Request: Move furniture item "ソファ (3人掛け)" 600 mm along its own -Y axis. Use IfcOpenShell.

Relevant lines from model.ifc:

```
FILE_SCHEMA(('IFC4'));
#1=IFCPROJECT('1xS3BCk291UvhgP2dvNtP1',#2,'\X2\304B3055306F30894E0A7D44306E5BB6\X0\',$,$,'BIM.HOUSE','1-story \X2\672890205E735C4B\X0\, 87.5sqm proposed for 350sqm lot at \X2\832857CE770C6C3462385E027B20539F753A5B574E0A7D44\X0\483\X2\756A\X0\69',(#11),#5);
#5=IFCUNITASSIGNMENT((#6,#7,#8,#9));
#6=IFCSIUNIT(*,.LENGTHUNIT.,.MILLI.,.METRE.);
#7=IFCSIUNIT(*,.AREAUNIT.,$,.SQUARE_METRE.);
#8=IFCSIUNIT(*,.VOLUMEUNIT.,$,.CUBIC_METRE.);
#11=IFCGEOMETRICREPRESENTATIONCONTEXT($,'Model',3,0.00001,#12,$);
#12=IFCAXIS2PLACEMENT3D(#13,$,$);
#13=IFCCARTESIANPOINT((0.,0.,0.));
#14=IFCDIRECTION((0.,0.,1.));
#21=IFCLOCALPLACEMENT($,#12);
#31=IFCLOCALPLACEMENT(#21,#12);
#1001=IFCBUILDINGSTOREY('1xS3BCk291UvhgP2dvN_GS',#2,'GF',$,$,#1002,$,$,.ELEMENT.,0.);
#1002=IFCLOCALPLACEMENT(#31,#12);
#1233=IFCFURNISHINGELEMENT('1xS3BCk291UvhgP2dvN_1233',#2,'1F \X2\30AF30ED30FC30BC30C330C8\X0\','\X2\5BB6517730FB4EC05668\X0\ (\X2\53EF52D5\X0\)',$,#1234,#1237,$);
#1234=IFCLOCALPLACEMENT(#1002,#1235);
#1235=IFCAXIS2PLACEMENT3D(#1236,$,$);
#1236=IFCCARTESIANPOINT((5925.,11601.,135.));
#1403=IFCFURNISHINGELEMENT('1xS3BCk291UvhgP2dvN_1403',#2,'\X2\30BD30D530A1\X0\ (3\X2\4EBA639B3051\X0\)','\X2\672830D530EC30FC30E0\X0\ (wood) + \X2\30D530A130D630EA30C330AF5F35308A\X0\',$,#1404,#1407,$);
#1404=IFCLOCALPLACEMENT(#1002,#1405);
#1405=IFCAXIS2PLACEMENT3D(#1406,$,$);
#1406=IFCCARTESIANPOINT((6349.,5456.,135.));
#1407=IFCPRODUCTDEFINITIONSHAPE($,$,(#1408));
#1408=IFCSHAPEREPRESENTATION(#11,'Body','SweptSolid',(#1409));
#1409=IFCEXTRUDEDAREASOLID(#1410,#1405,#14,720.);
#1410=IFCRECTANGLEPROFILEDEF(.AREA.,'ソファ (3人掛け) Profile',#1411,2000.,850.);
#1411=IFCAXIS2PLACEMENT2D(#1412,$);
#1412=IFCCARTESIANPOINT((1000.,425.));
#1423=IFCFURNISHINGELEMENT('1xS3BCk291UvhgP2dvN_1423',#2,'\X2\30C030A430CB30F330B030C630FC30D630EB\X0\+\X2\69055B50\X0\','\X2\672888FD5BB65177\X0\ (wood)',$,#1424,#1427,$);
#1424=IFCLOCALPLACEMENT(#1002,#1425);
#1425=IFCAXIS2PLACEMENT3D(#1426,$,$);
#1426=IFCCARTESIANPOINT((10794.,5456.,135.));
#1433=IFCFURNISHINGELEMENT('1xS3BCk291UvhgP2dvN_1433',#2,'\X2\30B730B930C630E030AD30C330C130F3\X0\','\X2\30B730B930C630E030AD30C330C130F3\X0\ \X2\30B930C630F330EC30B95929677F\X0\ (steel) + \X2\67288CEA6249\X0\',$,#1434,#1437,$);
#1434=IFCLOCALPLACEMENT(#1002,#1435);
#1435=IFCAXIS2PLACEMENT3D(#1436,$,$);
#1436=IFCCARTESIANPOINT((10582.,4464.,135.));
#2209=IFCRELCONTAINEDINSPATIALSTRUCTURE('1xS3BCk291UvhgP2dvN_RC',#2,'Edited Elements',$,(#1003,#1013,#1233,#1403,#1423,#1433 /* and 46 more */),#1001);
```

```python
import ifcopenshell
import ifcopenshell.api.geometry
import ifcopenshell.util.placement
import ifcopenshell.util.unit

model = ifcopenshell.open("model.ifc")
unit_scale = ifcopenshell.util.unit.calculate_unit_scale(model)

item = model.by_guid("1xS3BCk291UvhgP2dvN_1403")
matrix = ifcopenshell.util.placement.get_local_placement(item.ObjectPlacement)
matrix[:3, 3] -= matrix[:3, 1] * 0.6 / unit_scale
ifcopenshell.api.geometry.edit_object_placement(model, product=item, matrix=matrix, is_si=False)

print(ifcopenshell.util.placement.get_local_placement(item.ObjectPlacement).round(3) + 0.0)

model.write("model_v2.ifc")
```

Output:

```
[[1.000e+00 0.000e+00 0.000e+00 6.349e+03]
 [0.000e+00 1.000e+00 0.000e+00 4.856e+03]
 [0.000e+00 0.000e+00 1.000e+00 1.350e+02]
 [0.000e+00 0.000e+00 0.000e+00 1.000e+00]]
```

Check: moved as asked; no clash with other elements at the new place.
